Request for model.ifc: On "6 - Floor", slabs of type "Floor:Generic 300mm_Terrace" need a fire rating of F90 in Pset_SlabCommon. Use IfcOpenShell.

First a look at what the model holds.

```python
import ifcopenshell
import ifcopenshell.util.element

model = ifcopenshell.open("model.ifc")
print(model.schema)
storey = next(s for s in model.by_type("IfcBuildingStorey") if s.Name == "6 - Floor")
slabs = [e for e in ifcopenshell.util.element.get_decomposition(storey) if e.is_a("IfcSlab")]
seen = {}
for e in slabs:
    element_type = ifcopenshell.util.element.get_type(e)
    key = (element_type.Name if element_type != e and element_type else None, ifcopenshell.util.element.get_pset(e, "Pset_SlabCommon", "FireRating"))
    seen[key] = seen.get(key, 0) + 1
for (name, value), count in sorted(seen.items(), key=str):
    print(count, "x", name, "|", value)
```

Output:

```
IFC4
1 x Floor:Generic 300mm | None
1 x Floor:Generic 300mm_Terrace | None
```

```python
import ifcopenshell
import ifcopenshell.api.pset
import ifcopenshell.util.element

model = ifcopenshell.open("model.ifc")

storey = next(s for s in model.by_type("IfcBuildingStorey") if s.Name == "6 - Floor")
slabs = [e for e in ifcopenshell.util.element.get_decomposition(storey) if e.is_a("IfcSlab")]

count = 0
for e in slabs:
    element_type = ifcopenshell.util.element.get_type(e)
    if element_type in (None, e) or element_type.Name != "Floor:Generic 300mm_Terrace":
        continue
    # add_pset returns the element's existing set when there is one.
    pset = ifcopenshell.api.pset.add_pset(model, product=e, name="Pset_SlabCommon")
    ifcopenshell.api.pset.edit_pset(model, pset=pset, properties={"FireRating": "F90"})
    count += 1

print(count, "slabs updated")

model.write("model_rev.ifc")
```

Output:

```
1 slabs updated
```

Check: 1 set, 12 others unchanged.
